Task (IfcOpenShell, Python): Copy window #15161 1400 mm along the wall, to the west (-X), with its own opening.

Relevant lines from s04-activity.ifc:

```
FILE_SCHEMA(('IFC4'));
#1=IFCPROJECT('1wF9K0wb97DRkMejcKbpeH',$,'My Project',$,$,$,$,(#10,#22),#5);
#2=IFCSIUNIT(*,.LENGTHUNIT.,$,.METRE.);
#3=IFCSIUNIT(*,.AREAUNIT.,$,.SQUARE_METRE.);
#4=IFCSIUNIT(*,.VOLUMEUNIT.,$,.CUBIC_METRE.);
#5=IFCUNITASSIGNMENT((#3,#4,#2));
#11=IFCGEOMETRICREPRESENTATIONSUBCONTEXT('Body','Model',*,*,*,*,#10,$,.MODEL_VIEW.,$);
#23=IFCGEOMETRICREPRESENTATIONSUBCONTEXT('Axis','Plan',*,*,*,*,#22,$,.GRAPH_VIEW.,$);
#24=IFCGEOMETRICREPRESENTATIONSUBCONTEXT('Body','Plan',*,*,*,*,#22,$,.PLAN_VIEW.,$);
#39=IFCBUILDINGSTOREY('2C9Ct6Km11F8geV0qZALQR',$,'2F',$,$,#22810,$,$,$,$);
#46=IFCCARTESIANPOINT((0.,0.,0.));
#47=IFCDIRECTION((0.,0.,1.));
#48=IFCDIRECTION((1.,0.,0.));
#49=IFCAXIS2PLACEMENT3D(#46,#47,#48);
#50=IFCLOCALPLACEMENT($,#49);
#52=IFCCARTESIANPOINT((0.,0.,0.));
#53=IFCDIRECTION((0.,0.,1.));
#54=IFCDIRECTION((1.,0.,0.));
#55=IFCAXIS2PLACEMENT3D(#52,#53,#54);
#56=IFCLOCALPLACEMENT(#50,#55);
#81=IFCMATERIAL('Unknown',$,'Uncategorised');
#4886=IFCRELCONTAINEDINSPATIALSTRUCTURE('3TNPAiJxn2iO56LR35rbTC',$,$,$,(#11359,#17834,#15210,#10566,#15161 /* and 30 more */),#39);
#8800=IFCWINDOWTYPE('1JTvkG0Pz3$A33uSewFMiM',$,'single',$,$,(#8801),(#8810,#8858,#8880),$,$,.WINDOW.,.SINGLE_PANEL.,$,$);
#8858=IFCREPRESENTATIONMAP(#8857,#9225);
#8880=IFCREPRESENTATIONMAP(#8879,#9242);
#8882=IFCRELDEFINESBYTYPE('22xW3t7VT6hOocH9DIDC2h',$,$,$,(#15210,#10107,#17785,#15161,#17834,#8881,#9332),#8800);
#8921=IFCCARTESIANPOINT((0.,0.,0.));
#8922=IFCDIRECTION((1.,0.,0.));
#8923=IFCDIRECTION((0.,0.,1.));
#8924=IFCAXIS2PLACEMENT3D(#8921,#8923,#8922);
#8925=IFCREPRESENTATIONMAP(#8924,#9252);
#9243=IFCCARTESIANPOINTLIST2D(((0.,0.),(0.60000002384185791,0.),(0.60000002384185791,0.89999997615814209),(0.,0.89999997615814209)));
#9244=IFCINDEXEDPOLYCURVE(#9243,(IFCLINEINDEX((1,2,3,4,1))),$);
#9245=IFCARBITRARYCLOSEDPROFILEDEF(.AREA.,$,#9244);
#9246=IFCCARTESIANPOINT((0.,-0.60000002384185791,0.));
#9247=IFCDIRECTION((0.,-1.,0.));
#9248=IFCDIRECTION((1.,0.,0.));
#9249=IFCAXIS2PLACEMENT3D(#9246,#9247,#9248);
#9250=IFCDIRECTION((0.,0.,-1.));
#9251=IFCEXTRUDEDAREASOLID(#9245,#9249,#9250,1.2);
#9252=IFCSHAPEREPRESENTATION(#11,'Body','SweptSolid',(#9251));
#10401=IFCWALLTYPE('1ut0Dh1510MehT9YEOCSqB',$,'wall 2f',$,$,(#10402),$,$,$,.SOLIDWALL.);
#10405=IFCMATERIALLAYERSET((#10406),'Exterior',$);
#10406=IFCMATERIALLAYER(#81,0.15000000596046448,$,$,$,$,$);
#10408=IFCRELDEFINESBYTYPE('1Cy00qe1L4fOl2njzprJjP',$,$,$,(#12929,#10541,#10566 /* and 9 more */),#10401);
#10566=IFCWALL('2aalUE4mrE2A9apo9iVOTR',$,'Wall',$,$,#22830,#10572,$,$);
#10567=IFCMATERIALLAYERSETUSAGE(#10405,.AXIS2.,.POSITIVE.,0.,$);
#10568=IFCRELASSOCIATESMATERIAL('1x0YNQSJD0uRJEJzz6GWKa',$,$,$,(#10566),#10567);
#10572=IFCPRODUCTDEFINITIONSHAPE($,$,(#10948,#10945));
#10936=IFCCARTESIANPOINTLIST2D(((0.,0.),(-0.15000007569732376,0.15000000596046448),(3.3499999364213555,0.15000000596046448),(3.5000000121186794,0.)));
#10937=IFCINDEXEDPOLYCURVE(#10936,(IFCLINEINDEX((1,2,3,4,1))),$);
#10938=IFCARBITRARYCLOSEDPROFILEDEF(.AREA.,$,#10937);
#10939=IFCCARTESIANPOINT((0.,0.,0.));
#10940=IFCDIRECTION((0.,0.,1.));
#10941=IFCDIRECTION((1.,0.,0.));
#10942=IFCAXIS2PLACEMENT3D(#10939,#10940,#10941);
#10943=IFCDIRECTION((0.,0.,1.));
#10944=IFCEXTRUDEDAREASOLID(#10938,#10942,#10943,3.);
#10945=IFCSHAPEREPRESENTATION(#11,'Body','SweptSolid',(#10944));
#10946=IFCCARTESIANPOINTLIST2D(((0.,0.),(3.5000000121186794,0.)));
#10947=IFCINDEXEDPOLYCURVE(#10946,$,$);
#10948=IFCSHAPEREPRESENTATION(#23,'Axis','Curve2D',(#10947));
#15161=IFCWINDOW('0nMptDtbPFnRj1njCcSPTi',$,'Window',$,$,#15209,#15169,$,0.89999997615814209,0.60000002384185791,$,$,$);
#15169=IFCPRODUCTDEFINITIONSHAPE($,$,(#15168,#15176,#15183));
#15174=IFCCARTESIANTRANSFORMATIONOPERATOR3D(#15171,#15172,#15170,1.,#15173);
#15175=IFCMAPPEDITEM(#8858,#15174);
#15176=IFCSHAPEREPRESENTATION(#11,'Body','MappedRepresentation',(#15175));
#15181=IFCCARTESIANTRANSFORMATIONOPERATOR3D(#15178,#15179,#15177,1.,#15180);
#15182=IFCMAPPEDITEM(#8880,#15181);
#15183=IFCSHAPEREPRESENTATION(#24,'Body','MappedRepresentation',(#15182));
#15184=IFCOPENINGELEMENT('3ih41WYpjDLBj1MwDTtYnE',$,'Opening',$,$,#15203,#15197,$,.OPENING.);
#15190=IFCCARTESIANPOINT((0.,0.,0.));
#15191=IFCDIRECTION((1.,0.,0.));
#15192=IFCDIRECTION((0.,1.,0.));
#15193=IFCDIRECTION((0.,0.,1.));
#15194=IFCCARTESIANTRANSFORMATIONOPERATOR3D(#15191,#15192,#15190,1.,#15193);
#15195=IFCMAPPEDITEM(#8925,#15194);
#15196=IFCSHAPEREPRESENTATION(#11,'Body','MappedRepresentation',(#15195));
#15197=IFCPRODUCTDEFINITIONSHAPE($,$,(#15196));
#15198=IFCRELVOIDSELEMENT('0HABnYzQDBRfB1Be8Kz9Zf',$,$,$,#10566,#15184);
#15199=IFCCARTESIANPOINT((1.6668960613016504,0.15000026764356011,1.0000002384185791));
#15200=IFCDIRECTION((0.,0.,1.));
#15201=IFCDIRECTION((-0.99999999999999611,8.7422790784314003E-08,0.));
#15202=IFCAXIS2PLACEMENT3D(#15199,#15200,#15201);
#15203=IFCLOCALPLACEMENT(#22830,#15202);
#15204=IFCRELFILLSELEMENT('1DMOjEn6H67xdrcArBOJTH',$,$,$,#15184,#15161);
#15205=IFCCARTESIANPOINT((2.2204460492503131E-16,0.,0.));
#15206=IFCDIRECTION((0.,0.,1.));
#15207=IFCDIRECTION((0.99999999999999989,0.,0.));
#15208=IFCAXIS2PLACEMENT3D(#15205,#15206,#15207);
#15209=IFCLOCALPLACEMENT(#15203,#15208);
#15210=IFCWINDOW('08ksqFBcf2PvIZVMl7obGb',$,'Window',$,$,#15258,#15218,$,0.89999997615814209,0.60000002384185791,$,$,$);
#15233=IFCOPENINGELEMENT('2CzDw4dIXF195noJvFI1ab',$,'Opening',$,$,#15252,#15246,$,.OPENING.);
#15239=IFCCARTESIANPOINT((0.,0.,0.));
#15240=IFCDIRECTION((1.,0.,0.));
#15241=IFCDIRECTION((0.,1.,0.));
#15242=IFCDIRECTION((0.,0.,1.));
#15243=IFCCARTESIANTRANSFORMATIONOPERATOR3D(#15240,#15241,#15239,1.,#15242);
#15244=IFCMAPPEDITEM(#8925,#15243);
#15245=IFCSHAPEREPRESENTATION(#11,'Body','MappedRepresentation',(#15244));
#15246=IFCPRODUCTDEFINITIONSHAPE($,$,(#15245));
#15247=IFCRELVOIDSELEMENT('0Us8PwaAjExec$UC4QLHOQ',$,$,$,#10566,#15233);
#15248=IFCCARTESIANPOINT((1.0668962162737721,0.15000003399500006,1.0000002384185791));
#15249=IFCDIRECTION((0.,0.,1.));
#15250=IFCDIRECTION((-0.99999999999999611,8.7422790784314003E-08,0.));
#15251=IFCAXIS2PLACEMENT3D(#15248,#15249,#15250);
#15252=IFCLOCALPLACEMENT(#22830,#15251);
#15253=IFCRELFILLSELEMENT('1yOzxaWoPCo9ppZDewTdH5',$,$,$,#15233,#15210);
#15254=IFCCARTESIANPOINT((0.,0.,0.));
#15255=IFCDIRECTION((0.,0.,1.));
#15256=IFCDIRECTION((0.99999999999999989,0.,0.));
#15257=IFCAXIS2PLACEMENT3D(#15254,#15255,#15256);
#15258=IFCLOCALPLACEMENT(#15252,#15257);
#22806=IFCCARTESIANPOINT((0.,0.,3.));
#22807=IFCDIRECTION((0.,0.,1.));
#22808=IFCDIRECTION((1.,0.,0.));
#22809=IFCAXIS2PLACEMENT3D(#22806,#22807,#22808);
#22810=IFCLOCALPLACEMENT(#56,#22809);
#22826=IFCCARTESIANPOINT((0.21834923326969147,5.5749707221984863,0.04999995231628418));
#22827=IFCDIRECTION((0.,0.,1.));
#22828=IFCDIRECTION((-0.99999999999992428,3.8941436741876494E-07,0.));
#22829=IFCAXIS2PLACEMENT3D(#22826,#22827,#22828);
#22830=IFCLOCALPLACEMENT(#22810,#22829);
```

```python
import ifcopenshell
import ifcopenshell.api.feature
import ifcopenshell.api.geometry
import ifcopenshell.api.root
import ifcopenshell.geom
import ifcopenshell.util.element
import ifcopenshell.util.placement
import ifcopenshell.util.shape
import ifcopenshell.util.unit

model = ifcopenshell.open("s04-activity.ifc")
unit_scale = ifcopenshell.util.unit.calculate_unit_scale(model)
settings = ifcopenshell.geom.settings()


def volume(element):
    """Net volume in cubic metres, openings subtracted."""
    shape = ifcopenshell.geom.create_shape(settings, element)
    return ifcopenshell.util.shape.get_volume(shape.geometry)


window = model.by_id(15161)
opening = window.FillsVoids[0].RelatingOpeningElement
wall = opening.VoidsElements[0].RelatingBuildingElement
before = volume(wall)
shift = ifcopenshell.util.placement.get_local_placement(wall.ObjectPlacement)[:3, 0] * 1.4 / unit_scale

# copy_class copies the void relationship, type, container and properties, but no geometry.
new_opening = ifcopenshell.api.root.copy_class(model, product=opening)
new_opening.Representation = ifcopenshell.util.element.copy_deep(
    model, opening.Representation, exclude=["IfcGeometricRepresentationContext", "IfcRepresentationMap"]
)
new_window = ifcopenshell.api.root.copy_class(model, product=window)
new_window.Representation = ifcopenshell.util.element.copy_deep(
    model, window.Representation, exclude=["IfcGeometricRepresentationContext", "IfcRepresentationMap"]
)
ifcopenshell.api.feature.add_filling(model, opening=new_opening, element=new_window)

for old, new in ((opening, new_opening), (window, new_window)):
    matrix = ifcopenshell.util.placement.get_local_placement(old.ObjectPlacement)
    matrix[:3, 3] += shift
    ifcopenshell.api.geometry.edit_object_placement(model, product=new, matrix=matrix, is_si=False)

after = volume(wall)

print(f"wall volume {before:.3f} -> {after:.3f} m3")

model.write("s04-activity-out.ifc")
```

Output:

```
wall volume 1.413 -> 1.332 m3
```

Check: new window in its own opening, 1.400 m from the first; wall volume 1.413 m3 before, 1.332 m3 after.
